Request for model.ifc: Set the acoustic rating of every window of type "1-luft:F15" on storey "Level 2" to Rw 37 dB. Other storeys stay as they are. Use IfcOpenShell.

First a look at what the model holds.

```python
import ifcopenshell
import ifcopenshell.util.element

model = ifcopenshell.open("model.ifc")
print(model.schema)
storey = next(s for s in model.by_type("IfcBuildingStorey") if s.Name == "Level 2")
windows = [e for e in ifcopenshell.util.element.get_decomposition(storey) if e.is_a("IfcWindow")]
seen = {}
for e in windows:
    element_type = ifcopenshell.util.element.get_type(e)
    key = (element_type.Name if element_type != e and element_type else None, ifcopenshell.util.element.get_pset(e, "Pset_WindowCommon", "AcousticRating"))
    seen[key] = seen.get(key, 0) + 1
for (name, value), count in sorted(seen.items(), key=str):
    print(count, "x", name, "|", value)
```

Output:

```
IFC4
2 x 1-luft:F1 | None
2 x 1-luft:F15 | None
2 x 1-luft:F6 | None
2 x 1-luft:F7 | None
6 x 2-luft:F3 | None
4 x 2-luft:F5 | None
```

```python
import ifcopenshell
import ifcopenshell.api.pset
import ifcopenshell.util.element

model = ifcopenshell.open("model.ifc")

storey = next(s for s in model.by_type("IfcBuildingStorey") if s.Name == "Level 2")
windows = [e for e in ifcopenshell.util.element.get_decomposition(storey) if e.is_a("IfcWindow")]

count = 0
for e in windows:
    element_type = ifcopenshell.util.element.get_type(e)
    if element_type in (None, e) or element_type.Name != "1-luft:F15":
        continue
    # add_pset returns the element's existing set when there is one.
    pset = ifcopenshell.api.pset.add_pset(model, product=e, name="Pset_WindowCommon")
    ifcopenshell.api.pset.edit_pset(model, pset=pset, properties={"AcousticRating": "Rw 37 dB"})
    count += 1

print(count, "windows updated")

model.write("model_edited.ifc")
```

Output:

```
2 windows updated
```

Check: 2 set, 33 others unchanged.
